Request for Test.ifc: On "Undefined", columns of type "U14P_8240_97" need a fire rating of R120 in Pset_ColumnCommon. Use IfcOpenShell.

First a look at what the model holds.

```python
import ifcopenshell
import ifcopenshell.util.element

model = ifcopenshell.open("Test.ifc")
print(model.schema)
storey = next(s for s in model.by_type("IfcBuildingStorey") if s.Name == "Undefined")
columns = [e for e in ifcopenshell.util.element.get_decomposition(storey) if e.is_a("IfcColumn")]
seen = {}
for e in columns:
    element_type = ifcopenshell.util.element.get_type(e)
    key = (element_type.Name if element_type != e and element_type else None, ifcopenshell.util.element.get_pset(e, "Pset_ColumnCommon", "FireRating"))
    seen[key] = seen.get(key, 0) + 1
for (name, value), count in sorted(seen.items(), key=str):
    print(count, "x", name, "|", value)
```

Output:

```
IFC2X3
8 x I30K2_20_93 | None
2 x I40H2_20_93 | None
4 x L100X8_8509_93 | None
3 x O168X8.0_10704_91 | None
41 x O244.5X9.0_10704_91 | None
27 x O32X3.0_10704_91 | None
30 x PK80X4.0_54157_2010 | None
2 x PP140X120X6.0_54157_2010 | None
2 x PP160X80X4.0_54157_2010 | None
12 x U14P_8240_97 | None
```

```python
import ifcopenshell
import ifcopenshell.api.pset
import ifcopenshell.util.element

model = ifcopenshell.open("Test.ifc")

storey = next(s for s in model.by_type("IfcBuildingStorey") if s.Name == "Undefined")
columns = [e for e in ifcopenshell.util.element.get_decomposition(storey) if e.is_a("IfcColumn")]

count = 0
for e in columns:
    element_type = ifcopenshell.util.element.get_type(e)
    if element_type in (None, e) or element_type.Name != "U14P_8240_97":
        continue
    found = ifcopenshell.util.element.get_pset(e, "Pset_ColumnCommon", should_inherit=False)
    if found:
        pset = model.by_id(found["id"])
        if len(ifcopenshell.util.element.get_elements_by_pset(pset)) > 1:
            pset = ifcopenshell.api.pset.unshare_pset(model, products=[e], pset=pset)[0]
    else:
        pset = ifcopenshell.api.pset.add_pset(model, product=e, name="Pset_ColumnCommon")
    ifcopenshell.api.pset.edit_pset(model, pset=pset, properties={"FireRating": "R120"})
    count += 1

print(count, "columns updated")

model.write("Test_edited.ifc")
```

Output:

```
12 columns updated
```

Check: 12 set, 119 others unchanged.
